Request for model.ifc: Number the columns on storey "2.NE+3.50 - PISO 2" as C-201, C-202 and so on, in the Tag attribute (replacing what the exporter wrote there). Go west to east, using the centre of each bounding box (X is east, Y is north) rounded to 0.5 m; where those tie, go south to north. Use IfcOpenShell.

First a look at what the model holds.

```python
import ifcopenshell
import ifcopenshell.util.element
import ifcopenshell.util.placement

model = ifcopenshell.open("model.ifc")
print(model.schema)
storey = next(s for s in model.by_type("IfcBuildingStorey") if s.Name == "2.NE+3.50 - PISO 2")
columns = [e for e in ifcopenshell.util.element.get_decomposition(storey) if e.is_a("IfcColumn")]
for e in sorted(columns, key=lambda e: e.id()):
    origin = ifcopenshell.util.placement.get_local_placement(e.ObjectPlacement)[:3, 3]
    print(e.id(), e.Tag, e.Name, origin.round(2) + 0.0, sep=" | ")
```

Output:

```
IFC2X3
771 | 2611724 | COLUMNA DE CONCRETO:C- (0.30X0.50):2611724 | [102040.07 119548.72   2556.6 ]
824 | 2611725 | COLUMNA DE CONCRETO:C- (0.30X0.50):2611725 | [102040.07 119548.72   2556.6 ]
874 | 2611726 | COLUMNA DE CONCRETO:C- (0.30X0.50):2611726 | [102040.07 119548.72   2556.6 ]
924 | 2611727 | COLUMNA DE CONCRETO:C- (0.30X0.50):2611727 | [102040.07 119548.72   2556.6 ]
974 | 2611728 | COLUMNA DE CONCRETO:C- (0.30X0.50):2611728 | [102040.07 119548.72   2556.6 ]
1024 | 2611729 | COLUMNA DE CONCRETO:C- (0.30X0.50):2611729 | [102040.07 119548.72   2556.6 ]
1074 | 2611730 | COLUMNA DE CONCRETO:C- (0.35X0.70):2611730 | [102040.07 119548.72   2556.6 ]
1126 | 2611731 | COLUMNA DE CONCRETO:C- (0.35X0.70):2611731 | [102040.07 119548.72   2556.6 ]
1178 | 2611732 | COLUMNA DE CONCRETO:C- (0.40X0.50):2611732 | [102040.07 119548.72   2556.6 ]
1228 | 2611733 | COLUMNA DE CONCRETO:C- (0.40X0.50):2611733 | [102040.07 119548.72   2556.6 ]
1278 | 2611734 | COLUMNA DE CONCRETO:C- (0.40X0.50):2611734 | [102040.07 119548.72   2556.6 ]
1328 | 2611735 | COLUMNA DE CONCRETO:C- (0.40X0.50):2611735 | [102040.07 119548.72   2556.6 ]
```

```python
import ifcopenshell
import ifcopenshell.geom
import ifcopenshell.util.element
import ifcopenshell.util.shape

model = ifcopenshell.open("model.ifc")
settings = ifcopenshell.geom.settings()
settings.set("use-world-coords", True)


def centre(element):
    shape = ifcopenshell.geom.create_shape(settings, element)
    return ifcopenshell.util.shape.get_bbox_centroid(shape.geometry)


storey = next(s for s in model.by_type("IfcBuildingStorey") if s.Name == "2.NE+3.50 - PISO 2")
columns = [e for e in ifcopenshell.util.element.get_decomposition(storey) if e.is_a("IfcColumn")]

# Insertion points can sit at a corner or the storey origin, so sort by the geometry (in metres).
centres = {e: centre(e) for e in columns}
columns.sort(key=lambda e: (round(centres[e][0] / 0.5), centres[e][1]))

for i, e in enumerate(columns, start=1):
    number = f"C-2{i:02d}"
    e.Tag = number
    print(e.id(), number)

model.write("model-out.ifc")
```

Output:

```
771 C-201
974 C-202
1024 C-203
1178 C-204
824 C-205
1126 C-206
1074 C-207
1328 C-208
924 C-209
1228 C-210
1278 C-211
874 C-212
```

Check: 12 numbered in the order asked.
